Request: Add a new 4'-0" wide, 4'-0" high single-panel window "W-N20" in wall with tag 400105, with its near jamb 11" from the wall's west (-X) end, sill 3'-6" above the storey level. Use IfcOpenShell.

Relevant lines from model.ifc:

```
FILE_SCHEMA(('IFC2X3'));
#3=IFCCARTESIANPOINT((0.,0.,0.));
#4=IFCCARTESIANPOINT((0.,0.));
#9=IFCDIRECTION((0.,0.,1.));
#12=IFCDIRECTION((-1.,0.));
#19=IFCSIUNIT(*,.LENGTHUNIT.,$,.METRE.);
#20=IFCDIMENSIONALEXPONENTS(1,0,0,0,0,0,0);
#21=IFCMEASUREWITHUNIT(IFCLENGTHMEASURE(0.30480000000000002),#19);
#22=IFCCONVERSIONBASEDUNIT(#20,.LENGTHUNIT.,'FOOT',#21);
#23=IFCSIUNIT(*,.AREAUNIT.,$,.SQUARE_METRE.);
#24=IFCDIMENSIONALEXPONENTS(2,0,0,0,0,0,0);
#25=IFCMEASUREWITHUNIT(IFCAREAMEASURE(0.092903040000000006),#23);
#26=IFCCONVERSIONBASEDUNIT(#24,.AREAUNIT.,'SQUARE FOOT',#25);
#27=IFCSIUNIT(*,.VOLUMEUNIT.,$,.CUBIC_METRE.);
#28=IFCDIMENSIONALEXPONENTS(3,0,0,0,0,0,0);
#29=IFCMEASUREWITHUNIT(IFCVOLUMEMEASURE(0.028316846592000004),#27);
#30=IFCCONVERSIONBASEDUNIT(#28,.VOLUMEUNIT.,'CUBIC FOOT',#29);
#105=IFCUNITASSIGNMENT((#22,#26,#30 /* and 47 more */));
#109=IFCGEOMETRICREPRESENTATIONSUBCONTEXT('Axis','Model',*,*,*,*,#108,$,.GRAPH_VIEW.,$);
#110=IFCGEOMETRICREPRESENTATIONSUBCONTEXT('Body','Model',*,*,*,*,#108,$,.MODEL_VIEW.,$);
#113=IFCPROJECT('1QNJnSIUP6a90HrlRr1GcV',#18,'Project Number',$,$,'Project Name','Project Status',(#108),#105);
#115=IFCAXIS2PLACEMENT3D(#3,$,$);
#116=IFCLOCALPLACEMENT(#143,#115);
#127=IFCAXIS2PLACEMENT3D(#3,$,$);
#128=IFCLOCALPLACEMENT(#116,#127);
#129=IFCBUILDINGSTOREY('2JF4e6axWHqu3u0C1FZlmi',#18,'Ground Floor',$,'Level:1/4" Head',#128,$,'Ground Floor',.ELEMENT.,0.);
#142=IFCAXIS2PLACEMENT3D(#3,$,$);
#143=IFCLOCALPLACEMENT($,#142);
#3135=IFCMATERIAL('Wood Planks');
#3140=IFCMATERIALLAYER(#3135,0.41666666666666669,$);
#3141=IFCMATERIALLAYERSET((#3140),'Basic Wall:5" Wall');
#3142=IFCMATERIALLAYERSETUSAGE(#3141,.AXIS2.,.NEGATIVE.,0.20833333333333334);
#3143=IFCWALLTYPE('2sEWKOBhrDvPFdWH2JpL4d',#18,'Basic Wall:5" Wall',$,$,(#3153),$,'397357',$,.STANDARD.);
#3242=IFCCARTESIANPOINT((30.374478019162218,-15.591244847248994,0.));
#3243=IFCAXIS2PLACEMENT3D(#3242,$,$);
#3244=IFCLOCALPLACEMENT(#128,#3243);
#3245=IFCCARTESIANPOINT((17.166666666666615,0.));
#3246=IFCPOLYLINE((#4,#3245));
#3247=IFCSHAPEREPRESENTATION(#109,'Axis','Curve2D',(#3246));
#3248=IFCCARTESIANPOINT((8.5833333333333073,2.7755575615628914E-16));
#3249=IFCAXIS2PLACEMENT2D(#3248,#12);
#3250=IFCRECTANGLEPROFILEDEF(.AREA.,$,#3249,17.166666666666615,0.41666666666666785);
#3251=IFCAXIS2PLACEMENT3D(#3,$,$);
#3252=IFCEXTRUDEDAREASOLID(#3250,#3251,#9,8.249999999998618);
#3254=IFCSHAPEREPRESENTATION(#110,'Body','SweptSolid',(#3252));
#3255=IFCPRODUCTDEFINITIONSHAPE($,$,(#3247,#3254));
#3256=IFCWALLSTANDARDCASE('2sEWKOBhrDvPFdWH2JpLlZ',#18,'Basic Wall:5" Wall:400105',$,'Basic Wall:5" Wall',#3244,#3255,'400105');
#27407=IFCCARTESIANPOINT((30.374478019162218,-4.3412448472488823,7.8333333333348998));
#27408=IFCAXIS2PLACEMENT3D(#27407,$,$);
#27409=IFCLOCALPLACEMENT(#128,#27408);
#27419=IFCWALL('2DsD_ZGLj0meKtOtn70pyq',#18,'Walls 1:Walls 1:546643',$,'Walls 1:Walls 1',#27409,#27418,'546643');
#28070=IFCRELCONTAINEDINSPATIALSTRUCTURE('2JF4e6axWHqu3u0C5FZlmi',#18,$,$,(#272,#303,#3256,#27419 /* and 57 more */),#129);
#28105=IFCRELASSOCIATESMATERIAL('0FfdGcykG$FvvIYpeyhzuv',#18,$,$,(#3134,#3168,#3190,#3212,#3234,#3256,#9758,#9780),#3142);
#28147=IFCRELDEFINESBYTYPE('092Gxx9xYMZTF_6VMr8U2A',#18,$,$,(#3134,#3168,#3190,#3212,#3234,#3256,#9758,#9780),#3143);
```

```python
import numpy as np
import ifcopenshell
import ifcopenshell.api.feature
import ifcopenshell.api.geometry
import ifcopenshell.api.root
import ifcopenshell.api.spatial
import ifcopenshell.api.type
import ifcopenshell.geom
import ifcopenshell.util.element
import ifcopenshell.util.placement
import ifcopenshell.util.representation
import ifcopenshell.util.shape
import ifcopenshell.util.unit

model = ifcopenshell.open("model.ifc")
unit_scale = ifcopenshell.util.unit.calculate_unit_scale(model)
settings = ifcopenshell.geom.settings()


def volume(element):
    """Net volume in cubic metres, openings subtracted."""
    shape = ifcopenshell.geom.create_shape(settings, element)
    return ifcopenshell.util.shape.get_volume(shape.geometry)


wall = model.by_guid("2sEWKOBhrDvPFdWH2JpLlZ")
storey = ifcopenshell.util.element.get_container(wall, ifc_class="IfcBuildingStorey")
context = ifcopenshell.util.representation.get_context(model, "Model", "Body", "MODEL_VIEW")
before = volume(wall)

width, height, from_end, sill = 1.2192, 1.2192, 0.2794, 1.0668  # metres

# The wall runs along its own X axis, and the end named is its -X end.
wall_shape = ifcopenshell.geom.create_shape(settings, wall)
x, y, z = ifcopenshell.util.shape.get_vertices(wall_shape.geometry).T
start = x.min() + from_end
face, thickness = float(y.min()), float(y.max() - y.min())
wall_matrix = ifcopenshell.util.placement.get_local_placement(wall.ObjectPlacement)
level = ifcopenshell.util.placement.get_local_placement(storey.ObjectPlacement)[2, 3]


def in_wall(x, y):
    """Placement at x, y metres in the wall's axes, at sill height."""
    matrix = wall_matrix.copy()
    matrix[:, 3] = wall_matrix @ np.array([x / unit_scale, y / unit_scale, 0.0, 1.0])
    matrix[2, 3] = level + sill / unit_scale
    return matrix


# Opening: a box that overshoots both wall faces by 50 mm.
opening = ifcopenshell.api.root.create_entity(model, ifc_class="IfcOpeningElement")
box = ifcopenshell.api.geometry.add_wall_representation(
    model, context=context, length=width, height=height, thickness=thickness + 0.1
)
ifcopenshell.api.geometry.assign_representation(model, product=opening, representation=box)
ifcopenshell.api.geometry.edit_object_placement(model, product=opening, matrix=in_wall(start, face - 0.05), is_si=False)
ifcopenshell.api.feature.add_feature(model, feature=opening, element=wall)

window = ifcopenshell.api.root.create_entity(model, ifc_class="IfcWindow", name="W-N20")
window.OverallWidth, window.OverallHeight = width / unit_scale, height / unit_scale
body = ifcopenshell.api.geometry.add_window_representation(
    model,
    context=context,
    overall_width=window.OverallWidth,
    overall_height=window.OverallHeight,
    partition_type="SINGLE_PANEL",
)
ifcopenshell.api.geometry.assign_representation(model, product=window, representation=body)
ifcopenshell.api.spatial.assign_container(model, products=[window], relating_structure=storey)
fills = ifcopenshell.api.feature.add_filling(model, opening=opening, element=window)
fills.OwnerHistory = window.OwnerHistory  # required in IFC2X3

# IFC2X3 keeps the operation on the window style.
style = ifcopenshell.api.root.create_entity(model, ifc_class="IfcWindowStyle", name="W-N20")
style.OperationType, style.ConstructionType = "SINGLE_PANEL", "NOTDEFINED"
style.ParameterTakesPrecedence = style.Sizeable = False
ifcopenshell.api.type.assign_type(model, related_objects=[window], relating_type=style)

# Centre the window in the wall's thickness.
ifcopenshell.api.geometry.edit_object_placement(model, product=window, matrix=in_wall(start, face), is_si=False)
window_shape = ifcopenshell.geom.create_shape(settings, window)
depth = ifcopenshell.util.shape.get_vertices(window_shape.geometry)[:, 1]
offset = face + thickness / 2 - (depth.min() + depth.max()) / 2
ifcopenshell.api.geometry.edit_object_placement(model, product=window, matrix=in_wall(start, offset), is_si=False)

after = volume(wall)

print(f"wall volume {before:.3f} -> {after:.3f} m3")

model.write("model_updated.ifc")
```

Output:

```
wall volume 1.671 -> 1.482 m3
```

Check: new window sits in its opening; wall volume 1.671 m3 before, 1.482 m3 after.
